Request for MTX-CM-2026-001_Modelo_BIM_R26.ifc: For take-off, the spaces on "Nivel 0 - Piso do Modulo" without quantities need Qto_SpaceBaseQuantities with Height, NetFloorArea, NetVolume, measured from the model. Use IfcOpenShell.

First a look at what the model holds.

```python
import ifcopenshell
import ifcopenshell.util.element
import ifcopenshell.util.unit

model = ifcopenshell.open("MTX-CM-2026-001_Modelo_BIM_R26.ifc")
print(model.schema)
for unit_type in ("LENGTHUNIT", "AREAUNIT", "VOLUMEUNIT"):
    print(unit_type, ifcopenshell.util.unit.calculate_unit_scale(model, unit_type))
storey = next(s for s in model.by_type("IfcBuildingStorey") if s.Name == "Nivel 0 - Piso do Modulo")
spaces = [e for e in ifcopenshell.util.element.get_decomposition(storey) if e.is_a("IfcSpace")]
for e in sorted(spaces, key=lambda e: e.id()):
    print(e.id(), e.is_a(), e.Name, list(ifcopenshell.util.element.get_psets(e, qtos_only=True)), sep=" | ")
```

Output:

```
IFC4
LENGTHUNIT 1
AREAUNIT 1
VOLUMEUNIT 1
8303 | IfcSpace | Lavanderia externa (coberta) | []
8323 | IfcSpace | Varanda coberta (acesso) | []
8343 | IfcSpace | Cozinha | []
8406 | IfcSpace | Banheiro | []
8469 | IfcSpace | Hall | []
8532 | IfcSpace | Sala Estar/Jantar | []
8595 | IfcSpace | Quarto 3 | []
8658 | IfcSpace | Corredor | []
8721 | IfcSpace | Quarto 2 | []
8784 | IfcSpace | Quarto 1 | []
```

```python
import ifcopenshell
import ifcopenshell.api.pset
import ifcopenshell.geom
import ifcopenshell.util.element
import ifcopenshell.util.shape
import ifcopenshell.util.unit

model = ifcopenshell.open("MTX-CM-2026-001_Modelo_BIM_R26.ifc")
unit_scale = ifcopenshell.util.unit.calculate_unit_scale(model)
area_scale = ifcopenshell.util.unit.calculate_unit_scale(model, "AREAUNIT")
volume_scale = ifcopenshell.util.unit.calculate_unit_scale(model, "VOLUMEUNIT")
settings = ifcopenshell.geom.settings()

storey = next(s for s in model.by_type("IfcBuildingStorey") if s.Name == "Nivel 0 - Piso do Modulo")
spaces = [e for e in ifcopenshell.util.element.get_decomposition(storey) if e.is_a("IfcSpace")]

for e in sorted(spaces, key=lambda e: e.id()):
    if ifcopenshell.util.element.get_psets(e, qtos_only=True, should_inherit=False):
        continue
    # Geometry comes back in metres, in the element's own axes.
    shape = ifcopenshell.geom.create_shape(settings, e)
    values = {
        "Height": ifcopenshell.util.shape.get_z(shape.geometry) / unit_scale,
        "NetFloorArea": ifcopenshell.util.shape.get_footprint_area(shape.geometry) / area_scale,
        "NetVolume": ifcopenshell.util.shape.get_volume(shape.geometry) / volume_scale,
    }
    qto = ifcopenshell.api.pset.add_qto(model, product=e, name="Qto_SpaceBaseQuantities")
    ifcopenshell.api.pset.edit_qto(model, qto=qto, properties=values)
    print(e.id(), {k: round(v, 3) for k, v in values.items()})

model.write("MTX-CM-2026-001_Modelo_BIM_R26-out.ifc")
```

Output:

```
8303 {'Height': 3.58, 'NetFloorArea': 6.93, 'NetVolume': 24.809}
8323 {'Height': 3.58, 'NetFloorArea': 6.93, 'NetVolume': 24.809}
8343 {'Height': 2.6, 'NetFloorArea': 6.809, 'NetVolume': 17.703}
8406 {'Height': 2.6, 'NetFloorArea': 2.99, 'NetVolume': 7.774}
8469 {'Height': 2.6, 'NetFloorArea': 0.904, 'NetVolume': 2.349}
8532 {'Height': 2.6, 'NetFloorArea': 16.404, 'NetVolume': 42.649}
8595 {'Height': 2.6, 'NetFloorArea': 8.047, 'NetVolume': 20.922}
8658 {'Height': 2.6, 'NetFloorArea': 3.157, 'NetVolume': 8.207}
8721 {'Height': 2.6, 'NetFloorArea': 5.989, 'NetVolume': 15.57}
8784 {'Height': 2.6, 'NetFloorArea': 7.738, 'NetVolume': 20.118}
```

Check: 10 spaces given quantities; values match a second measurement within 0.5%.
